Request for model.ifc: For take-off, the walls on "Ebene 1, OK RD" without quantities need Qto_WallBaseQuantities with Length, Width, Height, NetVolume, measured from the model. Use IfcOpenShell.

First a look at what the model holds.

```python
import ifcopenshell
import ifcopenshell.util.element
import ifcopenshell.util.unit

model = ifcopenshell.open("model.ifc")
print(model.schema)
for unit_type in ("LENGTHUNIT", "AREAUNIT", "VOLUMEUNIT"):
    print(unit_type, ifcopenshell.util.unit.calculate_unit_scale(model, unit_type))
storey = next(s for s in model.by_type("IfcBuildingStorey") if s.Name == "Ebene 1, OK RD")
walls = [e for e in ifcopenshell.util.element.get_decomposition(storey) if e.is_a("IfcWall")]
for e in sorted(walls, key=lambda e: e.id()):
    print(e.id(), e.is_a(), e.Name, list(ifcopenshell.util.element.get_psets(e, qtos_only=True)), sep=" | ")
```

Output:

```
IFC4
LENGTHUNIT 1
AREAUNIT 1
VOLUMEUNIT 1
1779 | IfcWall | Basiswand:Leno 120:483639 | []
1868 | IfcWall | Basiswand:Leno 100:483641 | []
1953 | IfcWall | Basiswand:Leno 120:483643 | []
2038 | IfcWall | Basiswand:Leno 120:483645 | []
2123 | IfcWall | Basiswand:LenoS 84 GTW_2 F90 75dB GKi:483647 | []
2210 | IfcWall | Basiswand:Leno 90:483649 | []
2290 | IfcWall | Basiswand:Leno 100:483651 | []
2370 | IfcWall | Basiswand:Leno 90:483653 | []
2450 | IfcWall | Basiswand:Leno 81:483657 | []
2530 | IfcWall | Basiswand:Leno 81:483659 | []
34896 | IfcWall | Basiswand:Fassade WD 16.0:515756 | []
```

```python
import ifcopenshell
import ifcopenshell.api.pset
import ifcopenshell.geom
import ifcopenshell.util.element
import ifcopenshell.util.shape
import ifcopenshell.util.unit

model = ifcopenshell.open("model.ifc")
unit_scale = ifcopenshell.util.unit.calculate_unit_scale(model)
volume_scale = ifcopenshell.util.unit.calculate_unit_scale(model, "VOLUMEUNIT")
settings = ifcopenshell.geom.settings()

storey = next(s for s in model.by_type("IfcBuildingStorey") if s.Name == "Ebene 1, OK RD")
walls = [e for e in ifcopenshell.util.element.get_decomposition(storey) if e.is_a("IfcWall")]

for e in sorted(walls, key=lambda e: e.id()):
    if ifcopenshell.util.element.get_psets(e, qtos_only=True, should_inherit=False):
        continue
    # Geometry comes back in metres, in the element's own axes.
    shape = ifcopenshell.geom.create_shape(settings, e)
    values = {
        "Length": ifcopenshell.util.shape.get_x(shape.geometry) / unit_scale,
        "Width": ifcopenshell.util.shape.get_y(shape.geometry) / unit_scale,
        "Height": ifcopenshell.util.shape.get_z(shape.geometry) / unit_scale,
        "NetVolume": ifcopenshell.util.shape.get_volume(shape.geometry) / volume_scale,
    }
    qto = ifcopenshell.api.pset.add_qto(model, product=e, name="Qto_WallBaseQuantities")
    ifcopenshell.api.pset.edit_qto(model, qto=qto, properties=values)
    print(e.id(), {k: round(v, 3) for k, v in values.items()})

model.write("model_rev.ifc")
```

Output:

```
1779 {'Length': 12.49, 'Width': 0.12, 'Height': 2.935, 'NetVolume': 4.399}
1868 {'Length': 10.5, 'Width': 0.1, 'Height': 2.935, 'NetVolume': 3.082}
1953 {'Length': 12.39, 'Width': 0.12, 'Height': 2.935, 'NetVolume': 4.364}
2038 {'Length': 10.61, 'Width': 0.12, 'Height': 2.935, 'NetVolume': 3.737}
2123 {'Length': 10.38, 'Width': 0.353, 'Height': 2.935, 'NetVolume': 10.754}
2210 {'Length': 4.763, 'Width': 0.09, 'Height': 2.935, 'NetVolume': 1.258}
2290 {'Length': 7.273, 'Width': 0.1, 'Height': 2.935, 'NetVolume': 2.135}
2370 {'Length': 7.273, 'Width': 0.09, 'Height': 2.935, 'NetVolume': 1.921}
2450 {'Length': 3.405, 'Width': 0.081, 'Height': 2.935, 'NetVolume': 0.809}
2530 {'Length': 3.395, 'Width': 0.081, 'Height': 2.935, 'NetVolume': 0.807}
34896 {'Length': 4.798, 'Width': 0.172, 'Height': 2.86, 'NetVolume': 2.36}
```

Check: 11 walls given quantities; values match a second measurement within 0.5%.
